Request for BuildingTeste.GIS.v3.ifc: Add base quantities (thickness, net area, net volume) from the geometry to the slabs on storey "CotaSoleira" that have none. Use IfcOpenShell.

First a look at what the model holds.

```python
import ifcopenshell
import ifcopenshell.util.element
import ifcopenshell.util.unit

model = ifcopenshell.open("BuildingTeste.GIS.v3.ifc")
print(model.schema)
for unit_type in ("LENGTHUNIT", "AREAUNIT", "VOLUMEUNIT"):
    print(unit_type, ifcopenshell.util.unit.calculate_unit_scale(model, unit_type))
storey = next(s for s in model.by_type("IfcBuildingStorey") if s.Name == "CotaSoleira")
slabs = [e for e in ifcopenshell.util.element.get_decomposition(storey) if e.is_a("IfcSlab")]
for e in sorted(slabs, key=lambda e: e.id()):
    print(e.id(), e.is_a(), e.Name, list(ifcopenshell.util.element.get_psets(e, qtos_only=True)), sep=" | ")
```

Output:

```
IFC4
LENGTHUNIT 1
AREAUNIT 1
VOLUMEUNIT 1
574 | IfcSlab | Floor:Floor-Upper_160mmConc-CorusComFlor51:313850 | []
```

```python
import ifcopenshell
import ifcopenshell.api.pset
import ifcopenshell.geom
import ifcopenshell.util.element
import ifcopenshell.util.shape
import ifcopenshell.util.unit

model = ifcopenshell.open("BuildingTeste.GIS.v3.ifc")
unit_scale = ifcopenshell.util.unit.calculate_unit_scale(model)
area_scale = ifcopenshell.util.unit.calculate_unit_scale(model, "AREAUNIT")
volume_scale = ifcopenshell.util.unit.calculate_unit_scale(model, "VOLUMEUNIT")
settings = ifcopenshell.geom.settings()

storey = next(s for s in model.by_type("IfcBuildingStorey") if s.Name == "CotaSoleira")
slabs = [e for e in ifcopenshell.util.element.get_decomposition(storey) if e.is_a("IfcSlab")]

for e in sorted(slabs, key=lambda e: e.id()):
    if ifcopenshell.util.element.get_psets(e, qtos_only=True, should_inherit=False):
        continue
    # Geometry comes back in metres, in the element's own axes.
    shape = ifcopenshell.geom.create_shape(settings, e)
    values = {
        "Width": ifcopenshell.util.shape.get_z(shape.geometry) / unit_scale,
        "NetArea": ifcopenshell.util.shape.get_footprint_area(shape.geometry) / area_scale,
        "NetVolume": ifcopenshell.util.shape.get_volume(shape.geometry) / volume_scale,
    }
    qto = ifcopenshell.api.pset.add_qto(model, product=e, name="Qto_SlabBaseQuantities")
    ifcopenshell.api.pset.edit_qto(model, qto=qto, properties=values)
    print(e.id(), {k: round(v, 3) for k, v in values.items()})

model.write("BuildingTeste.GIS.v3_updated.ifc")
```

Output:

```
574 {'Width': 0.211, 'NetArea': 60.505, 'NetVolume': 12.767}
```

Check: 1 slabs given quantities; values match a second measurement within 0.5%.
